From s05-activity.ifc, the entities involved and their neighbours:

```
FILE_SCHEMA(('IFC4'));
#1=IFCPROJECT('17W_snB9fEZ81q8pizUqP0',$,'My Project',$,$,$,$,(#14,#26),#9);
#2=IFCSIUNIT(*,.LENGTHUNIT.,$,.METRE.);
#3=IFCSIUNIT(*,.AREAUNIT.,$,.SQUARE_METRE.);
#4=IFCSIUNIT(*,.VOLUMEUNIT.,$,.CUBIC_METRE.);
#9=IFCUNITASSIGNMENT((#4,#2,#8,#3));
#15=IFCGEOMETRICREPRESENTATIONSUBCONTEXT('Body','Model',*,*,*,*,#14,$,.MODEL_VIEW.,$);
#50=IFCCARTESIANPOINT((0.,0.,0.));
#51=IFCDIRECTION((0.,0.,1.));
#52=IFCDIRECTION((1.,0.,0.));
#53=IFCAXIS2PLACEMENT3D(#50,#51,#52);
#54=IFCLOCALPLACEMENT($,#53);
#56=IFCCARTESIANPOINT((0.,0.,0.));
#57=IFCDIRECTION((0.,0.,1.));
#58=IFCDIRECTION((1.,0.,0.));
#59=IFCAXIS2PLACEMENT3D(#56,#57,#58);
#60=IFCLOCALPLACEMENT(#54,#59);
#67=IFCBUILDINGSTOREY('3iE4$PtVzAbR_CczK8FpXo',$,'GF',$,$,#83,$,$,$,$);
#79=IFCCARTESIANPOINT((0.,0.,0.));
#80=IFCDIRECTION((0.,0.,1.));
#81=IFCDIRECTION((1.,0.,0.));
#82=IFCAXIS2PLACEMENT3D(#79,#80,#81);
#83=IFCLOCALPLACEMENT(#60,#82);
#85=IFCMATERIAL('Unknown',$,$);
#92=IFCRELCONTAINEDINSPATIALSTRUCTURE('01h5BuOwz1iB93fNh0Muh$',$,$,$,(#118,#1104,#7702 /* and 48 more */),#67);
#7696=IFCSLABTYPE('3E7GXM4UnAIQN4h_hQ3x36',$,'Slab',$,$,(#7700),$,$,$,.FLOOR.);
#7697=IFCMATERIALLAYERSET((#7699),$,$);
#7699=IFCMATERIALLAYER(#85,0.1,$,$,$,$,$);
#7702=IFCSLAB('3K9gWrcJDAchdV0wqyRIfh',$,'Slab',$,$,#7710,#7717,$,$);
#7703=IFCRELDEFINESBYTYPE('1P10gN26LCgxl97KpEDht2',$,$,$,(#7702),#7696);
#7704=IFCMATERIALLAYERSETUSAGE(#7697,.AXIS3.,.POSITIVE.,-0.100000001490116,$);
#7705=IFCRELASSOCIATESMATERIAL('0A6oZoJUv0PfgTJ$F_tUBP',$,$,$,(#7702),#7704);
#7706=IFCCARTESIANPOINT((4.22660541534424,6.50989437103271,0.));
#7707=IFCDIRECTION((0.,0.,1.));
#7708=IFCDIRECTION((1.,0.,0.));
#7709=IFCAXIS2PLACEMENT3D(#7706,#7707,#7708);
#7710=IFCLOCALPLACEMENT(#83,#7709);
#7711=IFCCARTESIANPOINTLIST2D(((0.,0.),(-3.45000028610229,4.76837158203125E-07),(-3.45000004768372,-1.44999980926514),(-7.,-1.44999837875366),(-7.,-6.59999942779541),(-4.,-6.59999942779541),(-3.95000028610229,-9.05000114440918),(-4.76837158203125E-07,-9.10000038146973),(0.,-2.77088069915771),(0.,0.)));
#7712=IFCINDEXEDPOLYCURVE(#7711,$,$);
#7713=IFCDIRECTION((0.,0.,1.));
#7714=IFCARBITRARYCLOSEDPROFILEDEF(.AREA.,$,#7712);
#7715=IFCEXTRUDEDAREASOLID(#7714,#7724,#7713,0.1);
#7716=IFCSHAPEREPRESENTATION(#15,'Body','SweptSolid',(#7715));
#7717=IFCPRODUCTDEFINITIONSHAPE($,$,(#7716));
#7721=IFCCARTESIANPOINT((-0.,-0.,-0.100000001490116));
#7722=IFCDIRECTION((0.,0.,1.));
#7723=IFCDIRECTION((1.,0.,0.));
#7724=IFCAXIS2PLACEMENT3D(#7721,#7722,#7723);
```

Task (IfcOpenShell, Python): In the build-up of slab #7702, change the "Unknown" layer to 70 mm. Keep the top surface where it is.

```python
import ifcopenshell
import ifcopenshell.util.element
import ifcopenshell.util.representation

model = ifcopenshell.open("s05-activity.ifc")

layer_set = model.by_id(7697)
layer = next(l for l in layer_set.MaterialLayers if l.Material and l.Material.Name == "Unknown")
change = 0.07 - layer.LayerThickness
layer.LayerThickness += change

# Geometry does not follow the layer set by itself.
slabs = [e for e in ifcopenshell.util.element.get_elements_by_material(model, layer_set) if e.is_a("IfcSlab")]
for slab in sorted(slabs, key=lambda e: e.id()):
    body = ifcopenshell.util.representation.get_representation(slab, "Model", "Body")
    solid = body.Items[0]
    old_depth = solid.Depth
    solid.Depth += change
    # Extruded upwards: lower the start of the extrusion so the top stays.
    x, y, z = solid.Position.Location.Coordinates
    solid.Position.Location = model.createIfcCartesianPoint((x, y, z - change))
    print(slab.id(), f"{old_depth:g} -> {solid.Depth:g}")

# The layers are counted up from the underside, which has moved.
for usage in {ifcopenshell.util.element.get_material(slab) for slab in slabs}:
    usage.OffsetFromReferenceLine -= change

model.write("s05-activity_edited.ifc")
```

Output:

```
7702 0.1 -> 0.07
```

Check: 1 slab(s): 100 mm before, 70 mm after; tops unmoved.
